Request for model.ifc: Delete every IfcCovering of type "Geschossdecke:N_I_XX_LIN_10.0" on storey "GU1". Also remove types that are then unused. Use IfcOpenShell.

First a look at what the model holds.

```python
import ifcopenshell
import ifcopenshell.util.element

model = ifcopenshell.open("model.ifc")
print(model.schema)
storey = next(s for s in model.by_type("IfcBuildingStorey") if s.Name == "GU1")
coverings = [e for e in ifcopenshell.util.element.get_decomposition(storey) if e.is_a("IfcCovering")]
seen = {}
for e in coverings:
    element_type = ifcopenshell.util.element.get_type(e)
    name = element_type.Name if element_type not in (None, e) else None
    seen[name] = seen.get(name, 0) + 1
for name, count in sorted(seen.items(), key=str):
    print(count, "x", name)
```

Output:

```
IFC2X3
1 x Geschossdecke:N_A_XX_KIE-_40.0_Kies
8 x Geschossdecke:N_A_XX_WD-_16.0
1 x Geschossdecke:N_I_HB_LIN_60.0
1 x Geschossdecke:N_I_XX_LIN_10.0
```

```python
import ifcopenshell
import ifcopenshell.api.root
import ifcopenshell.util.element

model = ifcopenshell.open("model.ifc")

storey = next(s for s in model.by_type("IfcBuildingStorey") if s.Name == "GU1")
coverings = [e for e in ifcopenshell.util.element.get_decomposition(storey) if e.is_a("IfcCovering")]
targets = [e for e in coverings if (t := ifcopenshell.util.element.get_type(e)) not in (None, e) and t.Name == "Geschossdecke:N_I_XX_LIN_10.0"]
types = {ifcopenshell.util.element.get_type(e) for e in targets} - {None, *targets}

for e in targets:
    ifcopenshell.api.root.remove_product(model, product=e)
print(len(targets), "removed")

unused = [t for t in types if not ifcopenshell.util.element.get_types(t)]
for t in unused:
    ifcopenshell.api.root.remove_product(model, product=t)
print(len(unused), "unused types removed")

model.write("model_edited.ifc")
```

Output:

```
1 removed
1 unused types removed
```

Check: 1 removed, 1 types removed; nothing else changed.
